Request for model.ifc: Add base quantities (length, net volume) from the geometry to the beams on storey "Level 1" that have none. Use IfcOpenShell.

First a look at what the model holds.

```python
import ifcopenshell
import ifcopenshell.util.element
import ifcopenshell.util.unit

model = ifcopenshell.open("model.ifc")
print(model.schema)
for unit_type in ("LENGTHUNIT", "AREAUNIT", "VOLUMEUNIT"):
    print(unit_type, ifcopenshell.util.unit.calculate_unit_scale(model, unit_type))
storey = next(s for s in model.by_type("IfcBuildingStorey") if s.Name == "Level 1")
beams = [e for e in ifcopenshell.util.element.get_decomposition(storey) if e.is_a("IfcBeam")]
for e in sorted(beams, key=lambda e: e.id()):
    print(e.id(), e.is_a(), e.Name, list(ifcopenshell.util.element.get_psets(e, qtos_only=True)), sep=" | ")
```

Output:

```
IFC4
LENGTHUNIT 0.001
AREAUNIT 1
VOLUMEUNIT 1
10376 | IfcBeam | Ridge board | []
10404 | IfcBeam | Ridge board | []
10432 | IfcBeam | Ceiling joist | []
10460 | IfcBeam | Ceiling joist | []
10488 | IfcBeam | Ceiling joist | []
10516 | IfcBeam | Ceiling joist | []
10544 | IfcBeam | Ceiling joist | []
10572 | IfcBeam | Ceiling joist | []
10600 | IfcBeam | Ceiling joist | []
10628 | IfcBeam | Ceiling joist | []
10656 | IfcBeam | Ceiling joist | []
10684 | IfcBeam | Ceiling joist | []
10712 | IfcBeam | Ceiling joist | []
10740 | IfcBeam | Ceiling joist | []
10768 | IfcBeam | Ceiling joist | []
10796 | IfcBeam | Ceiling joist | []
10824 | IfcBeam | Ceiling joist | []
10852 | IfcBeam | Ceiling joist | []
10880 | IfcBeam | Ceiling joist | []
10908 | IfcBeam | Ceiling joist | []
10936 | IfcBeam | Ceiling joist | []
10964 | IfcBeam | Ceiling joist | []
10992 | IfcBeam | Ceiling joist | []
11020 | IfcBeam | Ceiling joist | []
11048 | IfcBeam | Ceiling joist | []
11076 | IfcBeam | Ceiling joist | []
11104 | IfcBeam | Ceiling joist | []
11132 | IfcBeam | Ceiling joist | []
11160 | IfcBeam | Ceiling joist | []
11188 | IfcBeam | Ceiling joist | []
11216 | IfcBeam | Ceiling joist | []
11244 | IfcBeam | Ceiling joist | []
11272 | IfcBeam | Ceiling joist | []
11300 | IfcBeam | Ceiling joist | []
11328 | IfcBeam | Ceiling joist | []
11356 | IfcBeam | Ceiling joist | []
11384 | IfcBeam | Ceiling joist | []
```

```python
import ifcopenshell
import ifcopenshell.api.pset
import ifcopenshell.geom
import ifcopenshell.util.element
import ifcopenshell.util.shape
import ifcopenshell.util.unit

model = ifcopenshell.open("model.ifc")
unit_scale = ifcopenshell.util.unit.calculate_unit_scale(model)
volume_scale = ifcopenshell.util.unit.calculate_unit_scale(model, "VOLUMEUNIT")
settings = ifcopenshell.geom.settings()

storey = next(s for s in model.by_type("IfcBuildingStorey") if s.Name == "Level 1")
beams = [e for e in ifcopenshell.util.element.get_decomposition(storey) if e.is_a("IfcBeam")]

for e in sorted(beams, key=lambda e: e.id()):
    if ifcopenshell.util.element.get_psets(e, qtos_only=True, should_inherit=False):
        continue
    # Geometry comes back in metres, in the element's own axes.
    shape = ifcopenshell.geom.create_shape(settings, e)
    values = {
        "Length": ifcopenshell.util.shape.get_max_xyz(shape.geometry) / unit_scale,
        "NetVolume": ifcopenshell.util.shape.get_volume(shape.geometry) / volume_scale,
    }
    qto = ifcopenshell.api.pset.add_qto(model, product=e, name="Qto_BeamBaseQuantities")
    ifcopenshell.api.pset.edit_qto(model, qto=qto, properties=values)
    print(e.id(), {k: round(v, 3) for k, v in values.items()})

model.write("model_v2.ifc")
```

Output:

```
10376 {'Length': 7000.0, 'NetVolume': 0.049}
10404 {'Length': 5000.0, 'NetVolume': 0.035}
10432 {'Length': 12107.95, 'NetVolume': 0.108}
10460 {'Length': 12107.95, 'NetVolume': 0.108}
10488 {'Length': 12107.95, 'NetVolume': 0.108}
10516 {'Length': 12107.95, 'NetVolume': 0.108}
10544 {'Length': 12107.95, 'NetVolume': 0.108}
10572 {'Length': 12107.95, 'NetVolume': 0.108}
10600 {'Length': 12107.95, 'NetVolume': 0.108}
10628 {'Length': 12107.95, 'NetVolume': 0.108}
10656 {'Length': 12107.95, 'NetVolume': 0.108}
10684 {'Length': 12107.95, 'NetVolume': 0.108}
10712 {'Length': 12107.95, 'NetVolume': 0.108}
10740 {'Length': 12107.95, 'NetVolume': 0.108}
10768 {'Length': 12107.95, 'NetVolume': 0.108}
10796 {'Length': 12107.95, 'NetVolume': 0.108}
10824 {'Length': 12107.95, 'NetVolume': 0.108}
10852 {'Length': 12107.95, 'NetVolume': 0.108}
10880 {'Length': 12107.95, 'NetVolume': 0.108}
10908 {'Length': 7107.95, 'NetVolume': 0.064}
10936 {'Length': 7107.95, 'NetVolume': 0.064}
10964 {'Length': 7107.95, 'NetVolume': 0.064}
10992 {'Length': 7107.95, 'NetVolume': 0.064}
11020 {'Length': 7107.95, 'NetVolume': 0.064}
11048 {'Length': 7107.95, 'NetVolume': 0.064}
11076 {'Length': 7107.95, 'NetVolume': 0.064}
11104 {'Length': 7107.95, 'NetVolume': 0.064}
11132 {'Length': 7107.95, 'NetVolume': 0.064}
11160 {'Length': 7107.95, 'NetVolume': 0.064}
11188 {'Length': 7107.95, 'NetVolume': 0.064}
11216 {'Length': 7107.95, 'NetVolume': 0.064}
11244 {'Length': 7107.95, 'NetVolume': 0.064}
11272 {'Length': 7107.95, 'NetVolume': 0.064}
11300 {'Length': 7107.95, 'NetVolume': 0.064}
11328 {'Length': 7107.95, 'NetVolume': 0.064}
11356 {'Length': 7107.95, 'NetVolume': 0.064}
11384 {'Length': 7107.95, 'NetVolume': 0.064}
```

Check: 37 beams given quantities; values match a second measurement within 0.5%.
